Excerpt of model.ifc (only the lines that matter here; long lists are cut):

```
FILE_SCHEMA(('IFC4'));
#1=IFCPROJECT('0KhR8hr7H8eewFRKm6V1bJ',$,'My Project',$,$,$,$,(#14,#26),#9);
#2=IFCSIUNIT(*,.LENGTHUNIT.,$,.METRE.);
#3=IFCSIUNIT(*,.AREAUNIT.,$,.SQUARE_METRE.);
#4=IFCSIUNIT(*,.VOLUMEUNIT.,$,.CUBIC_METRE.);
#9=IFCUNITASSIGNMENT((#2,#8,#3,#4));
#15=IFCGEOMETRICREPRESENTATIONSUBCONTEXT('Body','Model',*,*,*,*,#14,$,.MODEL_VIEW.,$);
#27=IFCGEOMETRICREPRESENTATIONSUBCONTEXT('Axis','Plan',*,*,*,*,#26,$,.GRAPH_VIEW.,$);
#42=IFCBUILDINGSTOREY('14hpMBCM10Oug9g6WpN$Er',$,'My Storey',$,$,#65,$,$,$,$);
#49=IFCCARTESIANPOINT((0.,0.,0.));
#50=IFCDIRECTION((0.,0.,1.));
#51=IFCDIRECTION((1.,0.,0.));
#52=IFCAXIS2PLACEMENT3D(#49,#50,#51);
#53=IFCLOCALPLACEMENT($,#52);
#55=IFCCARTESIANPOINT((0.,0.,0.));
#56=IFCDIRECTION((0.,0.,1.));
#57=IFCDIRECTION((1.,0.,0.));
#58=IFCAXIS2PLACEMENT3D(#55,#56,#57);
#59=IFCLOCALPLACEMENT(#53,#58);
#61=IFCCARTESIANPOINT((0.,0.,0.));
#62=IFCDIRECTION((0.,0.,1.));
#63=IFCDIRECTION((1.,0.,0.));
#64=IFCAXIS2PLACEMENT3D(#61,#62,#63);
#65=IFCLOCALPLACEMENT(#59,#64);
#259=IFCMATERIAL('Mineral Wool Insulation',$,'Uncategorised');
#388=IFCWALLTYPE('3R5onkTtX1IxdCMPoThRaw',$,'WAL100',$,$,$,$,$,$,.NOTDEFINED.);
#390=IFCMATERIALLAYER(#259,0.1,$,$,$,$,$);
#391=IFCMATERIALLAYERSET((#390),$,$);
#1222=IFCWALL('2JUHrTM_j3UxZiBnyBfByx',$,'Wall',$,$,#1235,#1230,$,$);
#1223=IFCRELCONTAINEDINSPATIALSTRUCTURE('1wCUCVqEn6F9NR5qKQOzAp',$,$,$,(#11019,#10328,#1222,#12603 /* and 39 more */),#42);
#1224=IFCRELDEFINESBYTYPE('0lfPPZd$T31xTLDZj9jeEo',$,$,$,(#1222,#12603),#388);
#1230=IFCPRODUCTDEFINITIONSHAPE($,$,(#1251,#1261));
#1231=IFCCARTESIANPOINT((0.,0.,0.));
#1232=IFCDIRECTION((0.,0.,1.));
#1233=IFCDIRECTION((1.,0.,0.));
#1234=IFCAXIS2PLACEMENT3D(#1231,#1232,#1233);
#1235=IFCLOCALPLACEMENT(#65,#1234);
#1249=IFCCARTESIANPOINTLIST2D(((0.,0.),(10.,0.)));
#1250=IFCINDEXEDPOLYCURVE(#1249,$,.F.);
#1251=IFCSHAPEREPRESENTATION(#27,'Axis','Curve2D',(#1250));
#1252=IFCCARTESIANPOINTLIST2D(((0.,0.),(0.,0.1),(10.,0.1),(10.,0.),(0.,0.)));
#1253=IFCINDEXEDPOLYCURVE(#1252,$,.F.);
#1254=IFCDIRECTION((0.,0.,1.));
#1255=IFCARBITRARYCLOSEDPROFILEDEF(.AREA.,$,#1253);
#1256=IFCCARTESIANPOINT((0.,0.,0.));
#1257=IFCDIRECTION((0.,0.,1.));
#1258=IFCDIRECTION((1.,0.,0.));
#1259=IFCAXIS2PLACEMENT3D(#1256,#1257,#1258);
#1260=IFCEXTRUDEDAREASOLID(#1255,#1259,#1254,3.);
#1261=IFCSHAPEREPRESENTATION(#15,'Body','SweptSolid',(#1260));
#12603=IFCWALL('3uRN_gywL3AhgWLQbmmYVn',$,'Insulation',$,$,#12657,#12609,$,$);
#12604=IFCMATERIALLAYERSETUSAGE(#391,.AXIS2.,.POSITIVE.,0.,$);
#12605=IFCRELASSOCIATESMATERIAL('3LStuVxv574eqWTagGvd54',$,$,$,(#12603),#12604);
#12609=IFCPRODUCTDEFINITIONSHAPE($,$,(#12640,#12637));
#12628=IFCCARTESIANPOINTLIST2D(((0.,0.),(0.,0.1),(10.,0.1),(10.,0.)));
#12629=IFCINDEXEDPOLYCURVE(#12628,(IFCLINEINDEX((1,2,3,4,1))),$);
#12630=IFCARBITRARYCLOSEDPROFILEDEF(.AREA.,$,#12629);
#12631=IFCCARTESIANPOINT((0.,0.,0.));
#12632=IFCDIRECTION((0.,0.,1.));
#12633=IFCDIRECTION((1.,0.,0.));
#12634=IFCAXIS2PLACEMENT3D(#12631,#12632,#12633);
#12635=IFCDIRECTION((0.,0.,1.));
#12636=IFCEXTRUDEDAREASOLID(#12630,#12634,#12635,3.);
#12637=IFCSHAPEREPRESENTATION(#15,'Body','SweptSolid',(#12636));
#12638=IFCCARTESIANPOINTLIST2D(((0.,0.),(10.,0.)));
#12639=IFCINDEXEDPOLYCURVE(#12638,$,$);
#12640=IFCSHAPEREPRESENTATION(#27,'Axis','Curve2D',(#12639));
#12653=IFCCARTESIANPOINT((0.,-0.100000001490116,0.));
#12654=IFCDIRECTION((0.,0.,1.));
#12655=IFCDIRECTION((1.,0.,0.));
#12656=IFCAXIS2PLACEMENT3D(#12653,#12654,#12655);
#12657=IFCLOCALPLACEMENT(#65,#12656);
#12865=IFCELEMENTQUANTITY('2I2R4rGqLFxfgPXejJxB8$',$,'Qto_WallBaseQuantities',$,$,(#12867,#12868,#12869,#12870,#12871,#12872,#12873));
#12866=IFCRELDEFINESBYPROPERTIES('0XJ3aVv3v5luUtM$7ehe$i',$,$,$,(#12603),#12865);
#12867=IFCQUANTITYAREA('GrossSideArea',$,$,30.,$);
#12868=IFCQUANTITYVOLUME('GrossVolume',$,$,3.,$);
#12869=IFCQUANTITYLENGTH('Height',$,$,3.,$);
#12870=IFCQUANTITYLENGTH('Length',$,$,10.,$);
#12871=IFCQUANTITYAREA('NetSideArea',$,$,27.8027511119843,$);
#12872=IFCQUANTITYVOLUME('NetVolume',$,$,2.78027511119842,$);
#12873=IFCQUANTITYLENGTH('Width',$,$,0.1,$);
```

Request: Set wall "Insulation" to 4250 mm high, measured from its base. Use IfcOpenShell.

```python
import ifcopenshell
import ifcopenshell.api.pset
import ifcopenshell.geom
import ifcopenshell.util.element
import ifcopenshell.util.representation
import ifcopenshell.util.shape
import ifcopenshell.util.unit

model = ifcopenshell.open("model.ifc")
unit_scale = ifcopenshell.util.unit.calculate_unit_scale(model)
area_scale = ifcopenshell.util.unit.calculate_unit_scale(model, "AREAUNIT")
volume_scale = ifcopenshell.util.unit.calculate_unit_scale(model, "VOLUMEUNIT")
settings = ifcopenshell.geom.settings()


def volume(element):
    """Net volume in cubic metres, openings subtracted."""
    shape = ifcopenshell.geom.create_shape(settings, element)
    return ifcopenshell.util.shape.get_volume(shape.geometry)


wall = model.by_id(12603)
before = volume(wall)

body = ifcopenshell.util.representation.get_representation(wall, "Model", "Body")
solid = body.Items[0]
old_height = solid.Depth
solid.Depth = 4.25
after = volume(wall)
thickness = 0.1  # wall thickness in metres

# Update the stored height, areas and volumes.
qto = model.by_id(ifcopenshell.util.element.get_pset(wall, "Qto_WallBaseQuantities", should_inherit=False)["id"])
ifcopenshell.api.pset.edit_qto(model, qto=qto, properties={
    "GrossSideArea": ifcopenshell.util.element.get_pset(wall, "Qto_WallBaseQuantities", "GrossSideArea") * solid.Depth / old_height,
    "GrossVolume": ifcopenshell.util.element.get_pset(wall, "Qto_WallBaseQuantities", "GrossVolume") * solid.Depth / old_height,
    "Height": solid.Depth,
    "NetSideArea": after / thickness / area_scale,
    "NetVolume": after / volume_scale,
})

print(f"height {old_height:g} -> {solid.Depth:g}, volume {before:.3f} -> {after:.3f} m3")

model.write("model-out.ifc")
```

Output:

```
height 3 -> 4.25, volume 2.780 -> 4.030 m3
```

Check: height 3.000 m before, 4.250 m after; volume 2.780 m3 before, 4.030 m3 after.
